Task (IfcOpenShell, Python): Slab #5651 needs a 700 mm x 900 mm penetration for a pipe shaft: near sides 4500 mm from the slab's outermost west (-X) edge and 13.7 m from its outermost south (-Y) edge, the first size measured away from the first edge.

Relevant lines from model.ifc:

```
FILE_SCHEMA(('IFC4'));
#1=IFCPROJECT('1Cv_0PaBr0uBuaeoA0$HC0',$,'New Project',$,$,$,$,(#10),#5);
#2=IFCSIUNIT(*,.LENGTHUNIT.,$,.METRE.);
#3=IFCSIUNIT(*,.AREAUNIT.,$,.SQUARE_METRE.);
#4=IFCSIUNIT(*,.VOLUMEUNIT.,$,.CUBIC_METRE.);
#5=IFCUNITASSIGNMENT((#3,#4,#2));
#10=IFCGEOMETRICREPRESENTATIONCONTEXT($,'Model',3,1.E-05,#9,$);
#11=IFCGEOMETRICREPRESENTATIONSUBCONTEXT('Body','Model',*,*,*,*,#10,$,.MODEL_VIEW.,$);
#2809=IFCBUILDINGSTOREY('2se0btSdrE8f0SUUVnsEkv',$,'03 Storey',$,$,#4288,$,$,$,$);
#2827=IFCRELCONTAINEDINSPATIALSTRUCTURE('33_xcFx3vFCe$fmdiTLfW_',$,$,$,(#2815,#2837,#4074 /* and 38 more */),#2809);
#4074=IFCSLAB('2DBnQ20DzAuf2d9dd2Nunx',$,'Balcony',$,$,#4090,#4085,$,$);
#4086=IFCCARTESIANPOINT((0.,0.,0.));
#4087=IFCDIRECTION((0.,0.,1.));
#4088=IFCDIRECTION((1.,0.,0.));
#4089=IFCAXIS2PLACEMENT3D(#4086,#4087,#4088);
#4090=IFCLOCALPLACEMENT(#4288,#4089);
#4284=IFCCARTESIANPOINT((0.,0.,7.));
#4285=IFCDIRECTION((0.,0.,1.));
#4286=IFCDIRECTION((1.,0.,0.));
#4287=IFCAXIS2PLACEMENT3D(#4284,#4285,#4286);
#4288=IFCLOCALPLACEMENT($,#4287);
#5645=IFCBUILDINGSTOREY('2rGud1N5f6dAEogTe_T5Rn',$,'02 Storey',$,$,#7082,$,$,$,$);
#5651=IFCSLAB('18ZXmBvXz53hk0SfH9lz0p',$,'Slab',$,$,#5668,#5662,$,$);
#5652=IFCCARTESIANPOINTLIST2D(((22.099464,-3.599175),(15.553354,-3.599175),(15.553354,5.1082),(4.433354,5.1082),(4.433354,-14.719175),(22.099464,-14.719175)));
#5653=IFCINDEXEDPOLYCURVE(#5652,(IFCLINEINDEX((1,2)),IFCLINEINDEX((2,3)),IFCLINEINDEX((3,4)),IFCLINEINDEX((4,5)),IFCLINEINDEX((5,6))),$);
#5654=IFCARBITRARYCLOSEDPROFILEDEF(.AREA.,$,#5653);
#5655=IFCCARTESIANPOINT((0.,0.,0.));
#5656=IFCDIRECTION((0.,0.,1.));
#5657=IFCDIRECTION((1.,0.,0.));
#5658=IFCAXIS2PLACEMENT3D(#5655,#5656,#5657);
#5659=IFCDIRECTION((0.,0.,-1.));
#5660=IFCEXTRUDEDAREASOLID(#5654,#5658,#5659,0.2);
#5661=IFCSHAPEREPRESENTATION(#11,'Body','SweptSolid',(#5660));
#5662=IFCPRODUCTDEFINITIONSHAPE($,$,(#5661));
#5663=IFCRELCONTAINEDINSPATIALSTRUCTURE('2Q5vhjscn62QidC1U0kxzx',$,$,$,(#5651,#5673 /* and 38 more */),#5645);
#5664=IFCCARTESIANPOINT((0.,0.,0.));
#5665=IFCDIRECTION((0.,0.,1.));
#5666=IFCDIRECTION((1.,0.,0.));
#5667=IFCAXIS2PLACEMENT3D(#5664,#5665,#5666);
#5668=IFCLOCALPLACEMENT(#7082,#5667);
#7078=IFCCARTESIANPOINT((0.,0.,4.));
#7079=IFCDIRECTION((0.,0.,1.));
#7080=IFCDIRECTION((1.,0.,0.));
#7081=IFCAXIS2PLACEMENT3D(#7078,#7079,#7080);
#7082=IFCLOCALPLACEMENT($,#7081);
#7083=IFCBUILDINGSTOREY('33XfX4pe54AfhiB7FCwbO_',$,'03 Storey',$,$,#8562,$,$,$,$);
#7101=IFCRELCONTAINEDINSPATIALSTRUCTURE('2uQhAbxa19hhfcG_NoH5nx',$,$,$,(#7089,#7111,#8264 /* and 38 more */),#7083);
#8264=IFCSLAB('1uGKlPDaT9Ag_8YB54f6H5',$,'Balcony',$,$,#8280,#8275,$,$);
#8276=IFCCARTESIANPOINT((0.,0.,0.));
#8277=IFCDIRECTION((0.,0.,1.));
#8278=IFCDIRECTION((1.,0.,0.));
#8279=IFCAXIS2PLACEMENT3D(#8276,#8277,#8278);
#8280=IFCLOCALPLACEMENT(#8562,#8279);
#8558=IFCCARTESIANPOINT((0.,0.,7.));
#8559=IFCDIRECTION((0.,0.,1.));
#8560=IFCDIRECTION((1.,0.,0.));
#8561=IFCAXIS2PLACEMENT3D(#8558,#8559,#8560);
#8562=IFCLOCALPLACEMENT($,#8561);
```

```python
import numpy as np
import ifcopenshell
import ifcopenshell.api.feature
import ifcopenshell.api.geometry
import ifcopenshell.api.root
import ifcopenshell.geom
import ifcopenshell.util.placement
import ifcopenshell.util.representation
import ifcopenshell.util.shape
import ifcopenshell.util.unit

model = ifcopenshell.open("model.ifc")
unit_scale = ifcopenshell.util.unit.calculate_unit_scale(model)
settings = ifcopenshell.geom.settings()


def volume(element):
    """Net volume in cubic metres, openings subtracted."""
    shape = ifcopenshell.geom.create_shape(settings, element)
    return ifcopenshell.util.shape.get_volume(shape.geometry)


slab = model.by_guid("18ZXmBvXz53hk0SfH9lz0p")
before = volume(slab)

# Extent in the slab's own axes, in metres. The edges named are its -X and -Y sides.
slab_shape = ifcopenshell.geom.create_shape(settings, slab)
vertices = ifcopenshell.util.shape.get_vertices(slab_shape.geometry)
x_min, y_min, bottom = vertices.min(axis=0)
top = vertices[:, 2].max()

opening = ifcopenshell.api.root.create_entity(model, ifc_class="IfcOpeningElement", name="Pipe shaft opening", predefined_type="OPENING")
context = ifcopenshell.util.representation.get_context(model, "Model", "Body", "MODEL_VIEW")
width, depth = 0.7, 0.9
outline = [(0.0, 0.0), (width, 0.0), (width, depth), (0.0, depth), (0.0, 0.0)]
# Overshoot both faces by 50 mm so the cut is clean.
shape = ifcopenshell.api.geometry.add_slab_representation(
    model, context=context, depth=top - bottom + 0.1, polyline=outline
)
ifcopenshell.api.geometry.assign_representation(model, product=opening, representation=shape)

matrix = ifcopenshell.util.placement.get_local_placement(slab.ObjectPlacement)
matrix[:, 3] = matrix @ np.append(np.array([x_min + 4.5, y_min + 13.7, bottom - 0.05]) / unit_scale, 1.0)
ifcopenshell.api.geometry.edit_object_placement(model, product=opening, matrix=matrix, is_si=False)
ifcopenshell.api.feature.add_feature(model, feature=opening, element=slab)

after = volume(slab)

print(f"slab volume {before:.3f} -> {after:.3f} m3")

model.write("model_v2.ifc")
```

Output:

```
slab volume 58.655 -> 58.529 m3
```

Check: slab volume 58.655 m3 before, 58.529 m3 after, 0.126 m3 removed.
